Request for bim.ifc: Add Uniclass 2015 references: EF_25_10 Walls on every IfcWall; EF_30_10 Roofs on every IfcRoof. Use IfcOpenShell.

First a look at what the model holds.

```python
import ifcopenshell

model = ifcopenshell.open("bim.ifc")
print(model.schema)
print("classifications:", [c.Name for c in model.by_type("IfcClassification")])
for ifc_class in ("IfcDoor", "IfcRoof", "IfcStair", "IfcWall", "IfcWindow"):
    print(ifc_class, len(model.by_type(ifc_class)))
```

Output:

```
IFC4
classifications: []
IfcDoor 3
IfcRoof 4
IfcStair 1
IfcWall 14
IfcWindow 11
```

```python
import ifcopenshell
import ifcopenshell.api.classification

model = ifcopenshell.open("bim.ifc")

system = ifcopenshell.api.classification.add_classification(model, classification="Uniclass 2015")

codes = {
    "IfcWall": ("EF_25_10", "Walls"),
    "IfcRoof": ("EF_30_10", "Roofs"),
}
for ifc_class, (code, name) in codes.items():
    products = model.by_type(ifc_class)
    ifcopenshell.api.classification.add_reference(
        model, products=products, classification=system, identification=code, name=name
    )
    print(code, len(products))

model.write("bim-out.ifc")
```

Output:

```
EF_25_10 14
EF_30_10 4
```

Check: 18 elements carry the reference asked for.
